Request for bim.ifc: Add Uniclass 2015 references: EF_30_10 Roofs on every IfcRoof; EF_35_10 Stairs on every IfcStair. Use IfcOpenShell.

First a look at what the model holds.

```python
import ifcopenshell

model = ifcopenshell.open("bim.ifc")
print(model.schema)
print("classifications:", [c.Name for c in model.by_type("IfcClassification")])
for ifc_class in ("IfcDoor", "IfcRoof", "IfcStair", "IfcWall", "IfcWindow"):
    print(ifc_class, len(model.by_type(ifc_class)))
```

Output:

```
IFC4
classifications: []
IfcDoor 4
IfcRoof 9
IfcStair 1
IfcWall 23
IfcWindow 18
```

```python
import ifcopenshell
import ifcopenshell.api.classification

model = ifcopenshell.open("bim.ifc")

system = ifcopenshell.api.classification.add_classification(model, classification="Uniclass 2015")

codes = {
    "IfcRoof": ("EF_30_10", "Roofs"),
    "IfcStair": ("EF_35_10", "Stairs"),
}
for ifc_class, (code, name) in codes.items():
    products = model.by_type(ifc_class)
    ifcopenshell.api.classification.add_reference(
        model, products=products, classification=system, identification=code, name=name
    )
    print(code, len(products))

model.write("bim_v2.ifc")
```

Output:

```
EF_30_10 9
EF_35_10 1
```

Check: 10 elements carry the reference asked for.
